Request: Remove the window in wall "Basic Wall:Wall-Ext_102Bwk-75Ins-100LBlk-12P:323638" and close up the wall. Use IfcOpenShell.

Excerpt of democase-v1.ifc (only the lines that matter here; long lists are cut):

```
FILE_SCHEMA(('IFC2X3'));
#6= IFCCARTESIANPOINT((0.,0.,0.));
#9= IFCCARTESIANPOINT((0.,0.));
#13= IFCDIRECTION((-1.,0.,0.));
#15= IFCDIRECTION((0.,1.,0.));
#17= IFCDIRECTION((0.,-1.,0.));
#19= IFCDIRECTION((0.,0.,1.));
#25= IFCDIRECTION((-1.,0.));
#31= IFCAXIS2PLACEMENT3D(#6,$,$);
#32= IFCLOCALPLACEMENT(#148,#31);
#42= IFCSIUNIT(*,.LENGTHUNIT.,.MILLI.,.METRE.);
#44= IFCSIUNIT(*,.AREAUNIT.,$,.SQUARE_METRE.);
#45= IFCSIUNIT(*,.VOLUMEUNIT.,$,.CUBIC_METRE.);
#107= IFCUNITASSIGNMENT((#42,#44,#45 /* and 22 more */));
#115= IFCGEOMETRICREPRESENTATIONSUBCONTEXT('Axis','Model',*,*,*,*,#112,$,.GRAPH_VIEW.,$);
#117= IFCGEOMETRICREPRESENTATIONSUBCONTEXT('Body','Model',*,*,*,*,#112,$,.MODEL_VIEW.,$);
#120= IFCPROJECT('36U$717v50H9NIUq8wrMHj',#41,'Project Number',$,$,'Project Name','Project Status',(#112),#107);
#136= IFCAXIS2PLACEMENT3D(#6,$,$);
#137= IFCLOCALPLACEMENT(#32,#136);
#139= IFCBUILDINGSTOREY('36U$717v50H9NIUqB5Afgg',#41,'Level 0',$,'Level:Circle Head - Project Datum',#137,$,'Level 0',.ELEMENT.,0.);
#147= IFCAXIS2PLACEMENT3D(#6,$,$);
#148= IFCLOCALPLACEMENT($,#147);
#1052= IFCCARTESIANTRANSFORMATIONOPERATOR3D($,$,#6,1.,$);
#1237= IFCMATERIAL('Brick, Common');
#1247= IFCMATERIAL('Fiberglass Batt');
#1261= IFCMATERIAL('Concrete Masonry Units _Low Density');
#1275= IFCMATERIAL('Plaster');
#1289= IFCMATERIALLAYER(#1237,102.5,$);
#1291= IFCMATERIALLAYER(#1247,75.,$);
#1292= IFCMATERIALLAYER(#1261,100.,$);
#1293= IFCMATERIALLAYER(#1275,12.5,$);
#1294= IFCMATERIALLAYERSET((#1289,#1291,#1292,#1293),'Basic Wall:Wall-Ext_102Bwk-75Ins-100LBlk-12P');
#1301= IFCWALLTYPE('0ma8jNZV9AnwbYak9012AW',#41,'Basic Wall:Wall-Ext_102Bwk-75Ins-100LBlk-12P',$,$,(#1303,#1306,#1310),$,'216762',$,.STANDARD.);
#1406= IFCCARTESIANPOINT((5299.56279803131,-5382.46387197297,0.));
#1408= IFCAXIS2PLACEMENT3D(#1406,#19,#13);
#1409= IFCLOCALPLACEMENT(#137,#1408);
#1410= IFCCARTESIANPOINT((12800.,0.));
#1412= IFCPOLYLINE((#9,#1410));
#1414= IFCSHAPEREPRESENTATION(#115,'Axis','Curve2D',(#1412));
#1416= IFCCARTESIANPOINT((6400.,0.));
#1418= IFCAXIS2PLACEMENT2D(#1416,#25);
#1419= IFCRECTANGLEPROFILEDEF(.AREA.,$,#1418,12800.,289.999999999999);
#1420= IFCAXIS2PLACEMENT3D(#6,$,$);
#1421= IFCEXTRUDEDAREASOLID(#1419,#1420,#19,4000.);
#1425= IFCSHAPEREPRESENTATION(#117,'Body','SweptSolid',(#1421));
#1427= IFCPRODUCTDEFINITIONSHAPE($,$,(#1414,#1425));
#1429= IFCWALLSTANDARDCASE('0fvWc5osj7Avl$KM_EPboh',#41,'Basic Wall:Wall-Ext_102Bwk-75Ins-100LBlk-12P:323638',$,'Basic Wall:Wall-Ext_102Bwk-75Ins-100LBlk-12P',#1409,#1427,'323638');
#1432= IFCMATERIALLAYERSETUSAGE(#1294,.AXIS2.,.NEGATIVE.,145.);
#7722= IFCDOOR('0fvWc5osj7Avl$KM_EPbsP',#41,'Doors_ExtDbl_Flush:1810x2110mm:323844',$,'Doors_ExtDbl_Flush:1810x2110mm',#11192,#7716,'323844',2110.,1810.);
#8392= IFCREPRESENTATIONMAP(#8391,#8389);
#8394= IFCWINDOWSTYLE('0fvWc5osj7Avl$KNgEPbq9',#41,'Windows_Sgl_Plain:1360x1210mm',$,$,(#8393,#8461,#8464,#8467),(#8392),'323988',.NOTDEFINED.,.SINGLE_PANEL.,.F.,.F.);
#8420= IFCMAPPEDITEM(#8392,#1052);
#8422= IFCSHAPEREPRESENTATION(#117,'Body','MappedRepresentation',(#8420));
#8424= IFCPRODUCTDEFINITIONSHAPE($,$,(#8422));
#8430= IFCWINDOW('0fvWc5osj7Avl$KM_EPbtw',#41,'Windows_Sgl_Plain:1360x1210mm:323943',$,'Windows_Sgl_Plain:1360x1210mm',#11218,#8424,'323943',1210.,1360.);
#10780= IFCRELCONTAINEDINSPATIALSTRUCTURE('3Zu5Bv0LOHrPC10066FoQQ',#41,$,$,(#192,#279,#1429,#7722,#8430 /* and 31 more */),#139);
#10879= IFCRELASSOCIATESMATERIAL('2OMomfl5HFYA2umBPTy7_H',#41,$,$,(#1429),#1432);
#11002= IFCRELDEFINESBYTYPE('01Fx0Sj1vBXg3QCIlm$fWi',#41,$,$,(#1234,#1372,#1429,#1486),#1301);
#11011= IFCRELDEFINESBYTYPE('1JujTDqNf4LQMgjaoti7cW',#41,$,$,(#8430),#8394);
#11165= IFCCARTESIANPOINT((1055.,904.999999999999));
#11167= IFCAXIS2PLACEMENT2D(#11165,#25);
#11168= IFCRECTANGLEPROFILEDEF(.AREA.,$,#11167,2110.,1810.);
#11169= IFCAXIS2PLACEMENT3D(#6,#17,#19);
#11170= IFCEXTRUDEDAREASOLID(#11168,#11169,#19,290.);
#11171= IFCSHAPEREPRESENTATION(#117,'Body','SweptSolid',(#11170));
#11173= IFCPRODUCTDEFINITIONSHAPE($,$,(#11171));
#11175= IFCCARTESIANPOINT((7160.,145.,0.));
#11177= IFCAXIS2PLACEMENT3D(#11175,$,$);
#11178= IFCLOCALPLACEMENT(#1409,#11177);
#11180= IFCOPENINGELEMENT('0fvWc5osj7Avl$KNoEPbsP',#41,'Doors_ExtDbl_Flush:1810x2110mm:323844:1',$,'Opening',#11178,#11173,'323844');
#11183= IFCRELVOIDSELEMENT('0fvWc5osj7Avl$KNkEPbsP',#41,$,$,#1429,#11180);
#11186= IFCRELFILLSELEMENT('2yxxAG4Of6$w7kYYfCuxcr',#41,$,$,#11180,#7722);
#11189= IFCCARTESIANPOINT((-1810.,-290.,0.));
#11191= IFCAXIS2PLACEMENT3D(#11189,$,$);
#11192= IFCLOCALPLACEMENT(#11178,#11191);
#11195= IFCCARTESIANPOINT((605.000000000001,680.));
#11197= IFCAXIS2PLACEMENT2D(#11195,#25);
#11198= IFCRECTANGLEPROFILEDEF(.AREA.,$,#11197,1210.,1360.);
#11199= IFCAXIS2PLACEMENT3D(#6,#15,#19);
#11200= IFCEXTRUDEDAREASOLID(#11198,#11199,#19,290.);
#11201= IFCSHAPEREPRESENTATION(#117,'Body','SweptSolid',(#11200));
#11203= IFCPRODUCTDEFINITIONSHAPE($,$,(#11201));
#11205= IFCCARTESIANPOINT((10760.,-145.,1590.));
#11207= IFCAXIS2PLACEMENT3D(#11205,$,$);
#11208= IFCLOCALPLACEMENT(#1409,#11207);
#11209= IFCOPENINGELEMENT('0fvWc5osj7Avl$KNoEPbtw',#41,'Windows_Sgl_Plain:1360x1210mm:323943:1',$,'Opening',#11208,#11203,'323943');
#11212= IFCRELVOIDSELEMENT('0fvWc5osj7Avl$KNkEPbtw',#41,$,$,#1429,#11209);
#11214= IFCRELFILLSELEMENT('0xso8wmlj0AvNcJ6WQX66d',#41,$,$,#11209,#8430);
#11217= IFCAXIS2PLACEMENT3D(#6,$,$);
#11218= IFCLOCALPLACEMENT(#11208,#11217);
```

```python
import ifcopenshell
import ifcopenshell.api.feature
import ifcopenshell.api.root
import ifcopenshell.geom
import ifcopenshell.util.shape

model = ifcopenshell.open("democase-v1.ifc")
settings = ifcopenshell.geom.settings()


def volume(element):
    """Net volume in cubic metres, openings subtracted."""
    shape = ifcopenshell.geom.create_shape(settings, element)
    return ifcopenshell.util.shape.get_volume(shape.geometry)


window = model.by_guid("0fvWc5osj7Avl$KM_EPbtw")
opening = window.FillsVoids[0].RelatingOpeningElement
wall = opening.VoidsElements[0].RelatingBuildingElement
before = volume(wall)

ifcopenshell.api.root.remove_product(model, product=window)
ifcopenshell.api.feature.remove_feature(model, feature=opening)

after = volume(wall)

print(f"wall volume {before:.3f} -> {after:.3f} m3")

model.write("democase-v1-out.ifc")
```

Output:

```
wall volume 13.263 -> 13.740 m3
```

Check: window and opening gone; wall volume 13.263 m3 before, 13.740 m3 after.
